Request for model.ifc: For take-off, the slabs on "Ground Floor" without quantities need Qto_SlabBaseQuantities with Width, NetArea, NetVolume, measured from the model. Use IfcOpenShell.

First a look at what the model holds.

```python
import ifcopenshell
import ifcopenshell.util.element
import ifcopenshell.util.unit

model = ifcopenshell.open("model.ifc")
print(model.schema)
for unit_type in ("LENGTHUNIT", "AREAUNIT", "VOLUMEUNIT"):
    print(unit_type, ifcopenshell.util.unit.calculate_unit_scale(model, unit_type))
storey = next(s for s in model.by_type("IfcBuildingStorey") if s.Name == "Ground Floor")
slabs = [e for e in ifcopenshell.util.element.get_decomposition(storey) if e.is_a("IfcSlab")]
for e in sorted(slabs, key=lambda e: e.id()):
    print(e.id(), e.is_a(), e.Name, list(ifcopenshell.util.element.get_psets(e, qtos_only=True)), sep=" | ")
```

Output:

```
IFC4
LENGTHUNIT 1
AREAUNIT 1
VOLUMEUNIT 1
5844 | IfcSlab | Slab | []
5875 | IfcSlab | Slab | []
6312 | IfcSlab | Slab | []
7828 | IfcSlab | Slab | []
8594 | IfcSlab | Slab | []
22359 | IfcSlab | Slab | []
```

```python
import ifcopenshell
import ifcopenshell.api.pset
import ifcopenshell.geom
import ifcopenshell.util.element
import ifcopenshell.util.shape
import ifcopenshell.util.unit

model = ifcopenshell.open("model.ifc")
unit_scale = ifcopenshell.util.unit.calculate_unit_scale(model)
area_scale = ifcopenshell.util.unit.calculate_unit_scale(model, "AREAUNIT")
volume_scale = ifcopenshell.util.unit.calculate_unit_scale(model, "VOLUMEUNIT")
settings = ifcopenshell.geom.settings()

storey = next(s for s in model.by_type("IfcBuildingStorey") if s.Name == "Ground Floor")
slabs = [e for e in ifcopenshell.util.element.get_decomposition(storey) if e.is_a("IfcSlab")]

for e in sorted(slabs, key=lambda e: e.id()):
    if ifcopenshell.util.element.get_psets(e, qtos_only=True, should_inherit=False):
        continue
    # Geometry comes back in metres, in the element's own axes.
    shape = ifcopenshell.geom.create_shape(settings, e)
    values = {
        "Width": ifcopenshell.util.shape.get_z(shape.geometry) / unit_scale,
        "NetArea": ifcopenshell.util.shape.get_footprint_area(shape.geometry) / area_scale,
        "NetVolume": ifcopenshell.util.shape.get_volume(shape.geometry) / volume_scale,
    }
    qto = ifcopenshell.api.pset.add_qto(model, product=e, name="Qto_SlabBaseQuantities")
    ifcopenshell.api.pset.edit_qto(model, qto=qto, properties=values)
    print(e.id(), {k: round(v, 3) for k, v in values.items()})

model.write("model_edited.ifc")
```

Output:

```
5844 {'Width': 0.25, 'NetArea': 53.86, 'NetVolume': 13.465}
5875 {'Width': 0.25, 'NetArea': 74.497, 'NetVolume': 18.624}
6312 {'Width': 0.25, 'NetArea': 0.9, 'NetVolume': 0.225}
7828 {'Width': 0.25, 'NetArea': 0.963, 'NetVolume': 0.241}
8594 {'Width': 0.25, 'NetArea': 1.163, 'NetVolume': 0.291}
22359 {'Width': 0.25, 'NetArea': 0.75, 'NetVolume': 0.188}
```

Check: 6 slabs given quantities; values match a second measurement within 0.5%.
